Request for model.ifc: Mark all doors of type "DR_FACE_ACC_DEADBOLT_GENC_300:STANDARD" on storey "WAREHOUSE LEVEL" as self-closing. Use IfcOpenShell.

First a look at what the model holds.

```python
import ifcopenshell
import ifcopenshell.util.element

model = ifcopenshell.open("model.ifc")
print(model.schema)
storey = next(s for s in model.by_type("IfcBuildingStorey") if s.Name == "WAREHOUSE LEVEL")
doors = [e for e in ifcopenshell.util.element.get_decomposition(storey) if e.is_a("IfcDoor")]
seen = {}
for e in doors:
    element_type = ifcopenshell.util.element.get_type(e)
    key = (element_type.Name if element_type != e and element_type else None, ifcopenshell.util.element.get_pset(e, "Pset_DoorCommon", "SelfClosing"))
    seen[key] = seen.get(key, 0) + 1
for (name, value), count in sorted(seen.items(), key=str):
    print(count, "x", name, "|", value)
```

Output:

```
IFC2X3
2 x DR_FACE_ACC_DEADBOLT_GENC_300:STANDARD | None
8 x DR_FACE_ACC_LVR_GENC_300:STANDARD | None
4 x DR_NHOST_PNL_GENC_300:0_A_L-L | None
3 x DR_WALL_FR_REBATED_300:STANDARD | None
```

```python
import ifcopenshell
import ifcopenshell.api.pset
import ifcopenshell.util.element

model = ifcopenshell.open("model.ifc")

storey = next(s for s in model.by_type("IfcBuildingStorey") if s.Name == "WAREHOUSE LEVEL")
doors = [e for e in ifcopenshell.util.element.get_decomposition(storey) if e.is_a("IfcDoor")]

count = 0
for e in doors:
    element_type = ifcopenshell.util.element.get_type(e)
    if element_type in (None, e) or element_type.Name != "DR_FACE_ACC_DEADBOLT_GENC_300:STANDARD":
        continue
    # add_pset returns the element's existing set when there is one.
    pset = ifcopenshell.api.pset.add_pset(model, product=e, name="Pset_DoorCommon")
    ifcopenshell.api.pset.edit_pset(model, pset=pset, properties={"SelfClosing": True})
    count += 1

print(count, "doors updated")

model.write("model_v2.ifc")
```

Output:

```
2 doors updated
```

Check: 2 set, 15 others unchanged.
